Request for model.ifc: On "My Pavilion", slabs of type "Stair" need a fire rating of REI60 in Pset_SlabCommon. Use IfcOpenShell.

First a look at what the model holds.

```python
import ifcopenshell
import ifcopenshell.util.element

model = ifcopenshell.open("model.ifc")
print(model.schema)
storey = next(s for s in model.by_type("IfcBuildingStorey") if s.Name == "My Pavilion")
slabs = [e for e in ifcopenshell.util.element.get_decomposition(storey) if e.is_a("IfcSlab")]
seen = {}
for e in slabs:
    element_type = ifcopenshell.util.element.get_type(e)
    key = (element_type.Name if element_type != e and element_type else None, ifcopenshell.util.element.get_pset(e, "Pset_SlabCommon", "FireRating"))
    seen[key] = seen.get(key, 0) + 1
for (name, value), count in sorted(seen.items(), key=str):
    print(count, "x", name, "|", value)
```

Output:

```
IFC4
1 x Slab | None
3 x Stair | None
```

```python
import ifcopenshell
import ifcopenshell.api.pset
import ifcopenshell.util.element

model = ifcopenshell.open("model.ifc")

storey = next(s for s in model.by_type("IfcBuildingStorey") if s.Name == "My Pavilion")
slabs = [e for e in ifcopenshell.util.element.get_decomposition(storey) if e.is_a("IfcSlab")]

count = 0
for e in slabs:
    element_type = ifcopenshell.util.element.get_type(e)
    if element_type in (None, e) or element_type.Name != "Stair":
        continue
    # add_pset returns the element's existing set when there is one.
    pset = ifcopenshell.api.pset.add_pset(model, product=e, name="Pset_SlabCommon")
    ifcopenshell.api.pset.edit_pset(model, pset=pset, properties={"FireRating": "REI60"})
    count += 1

print(count, "slabs updated")

model.write("model_rev.ifc")
```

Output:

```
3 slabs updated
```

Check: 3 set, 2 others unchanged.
